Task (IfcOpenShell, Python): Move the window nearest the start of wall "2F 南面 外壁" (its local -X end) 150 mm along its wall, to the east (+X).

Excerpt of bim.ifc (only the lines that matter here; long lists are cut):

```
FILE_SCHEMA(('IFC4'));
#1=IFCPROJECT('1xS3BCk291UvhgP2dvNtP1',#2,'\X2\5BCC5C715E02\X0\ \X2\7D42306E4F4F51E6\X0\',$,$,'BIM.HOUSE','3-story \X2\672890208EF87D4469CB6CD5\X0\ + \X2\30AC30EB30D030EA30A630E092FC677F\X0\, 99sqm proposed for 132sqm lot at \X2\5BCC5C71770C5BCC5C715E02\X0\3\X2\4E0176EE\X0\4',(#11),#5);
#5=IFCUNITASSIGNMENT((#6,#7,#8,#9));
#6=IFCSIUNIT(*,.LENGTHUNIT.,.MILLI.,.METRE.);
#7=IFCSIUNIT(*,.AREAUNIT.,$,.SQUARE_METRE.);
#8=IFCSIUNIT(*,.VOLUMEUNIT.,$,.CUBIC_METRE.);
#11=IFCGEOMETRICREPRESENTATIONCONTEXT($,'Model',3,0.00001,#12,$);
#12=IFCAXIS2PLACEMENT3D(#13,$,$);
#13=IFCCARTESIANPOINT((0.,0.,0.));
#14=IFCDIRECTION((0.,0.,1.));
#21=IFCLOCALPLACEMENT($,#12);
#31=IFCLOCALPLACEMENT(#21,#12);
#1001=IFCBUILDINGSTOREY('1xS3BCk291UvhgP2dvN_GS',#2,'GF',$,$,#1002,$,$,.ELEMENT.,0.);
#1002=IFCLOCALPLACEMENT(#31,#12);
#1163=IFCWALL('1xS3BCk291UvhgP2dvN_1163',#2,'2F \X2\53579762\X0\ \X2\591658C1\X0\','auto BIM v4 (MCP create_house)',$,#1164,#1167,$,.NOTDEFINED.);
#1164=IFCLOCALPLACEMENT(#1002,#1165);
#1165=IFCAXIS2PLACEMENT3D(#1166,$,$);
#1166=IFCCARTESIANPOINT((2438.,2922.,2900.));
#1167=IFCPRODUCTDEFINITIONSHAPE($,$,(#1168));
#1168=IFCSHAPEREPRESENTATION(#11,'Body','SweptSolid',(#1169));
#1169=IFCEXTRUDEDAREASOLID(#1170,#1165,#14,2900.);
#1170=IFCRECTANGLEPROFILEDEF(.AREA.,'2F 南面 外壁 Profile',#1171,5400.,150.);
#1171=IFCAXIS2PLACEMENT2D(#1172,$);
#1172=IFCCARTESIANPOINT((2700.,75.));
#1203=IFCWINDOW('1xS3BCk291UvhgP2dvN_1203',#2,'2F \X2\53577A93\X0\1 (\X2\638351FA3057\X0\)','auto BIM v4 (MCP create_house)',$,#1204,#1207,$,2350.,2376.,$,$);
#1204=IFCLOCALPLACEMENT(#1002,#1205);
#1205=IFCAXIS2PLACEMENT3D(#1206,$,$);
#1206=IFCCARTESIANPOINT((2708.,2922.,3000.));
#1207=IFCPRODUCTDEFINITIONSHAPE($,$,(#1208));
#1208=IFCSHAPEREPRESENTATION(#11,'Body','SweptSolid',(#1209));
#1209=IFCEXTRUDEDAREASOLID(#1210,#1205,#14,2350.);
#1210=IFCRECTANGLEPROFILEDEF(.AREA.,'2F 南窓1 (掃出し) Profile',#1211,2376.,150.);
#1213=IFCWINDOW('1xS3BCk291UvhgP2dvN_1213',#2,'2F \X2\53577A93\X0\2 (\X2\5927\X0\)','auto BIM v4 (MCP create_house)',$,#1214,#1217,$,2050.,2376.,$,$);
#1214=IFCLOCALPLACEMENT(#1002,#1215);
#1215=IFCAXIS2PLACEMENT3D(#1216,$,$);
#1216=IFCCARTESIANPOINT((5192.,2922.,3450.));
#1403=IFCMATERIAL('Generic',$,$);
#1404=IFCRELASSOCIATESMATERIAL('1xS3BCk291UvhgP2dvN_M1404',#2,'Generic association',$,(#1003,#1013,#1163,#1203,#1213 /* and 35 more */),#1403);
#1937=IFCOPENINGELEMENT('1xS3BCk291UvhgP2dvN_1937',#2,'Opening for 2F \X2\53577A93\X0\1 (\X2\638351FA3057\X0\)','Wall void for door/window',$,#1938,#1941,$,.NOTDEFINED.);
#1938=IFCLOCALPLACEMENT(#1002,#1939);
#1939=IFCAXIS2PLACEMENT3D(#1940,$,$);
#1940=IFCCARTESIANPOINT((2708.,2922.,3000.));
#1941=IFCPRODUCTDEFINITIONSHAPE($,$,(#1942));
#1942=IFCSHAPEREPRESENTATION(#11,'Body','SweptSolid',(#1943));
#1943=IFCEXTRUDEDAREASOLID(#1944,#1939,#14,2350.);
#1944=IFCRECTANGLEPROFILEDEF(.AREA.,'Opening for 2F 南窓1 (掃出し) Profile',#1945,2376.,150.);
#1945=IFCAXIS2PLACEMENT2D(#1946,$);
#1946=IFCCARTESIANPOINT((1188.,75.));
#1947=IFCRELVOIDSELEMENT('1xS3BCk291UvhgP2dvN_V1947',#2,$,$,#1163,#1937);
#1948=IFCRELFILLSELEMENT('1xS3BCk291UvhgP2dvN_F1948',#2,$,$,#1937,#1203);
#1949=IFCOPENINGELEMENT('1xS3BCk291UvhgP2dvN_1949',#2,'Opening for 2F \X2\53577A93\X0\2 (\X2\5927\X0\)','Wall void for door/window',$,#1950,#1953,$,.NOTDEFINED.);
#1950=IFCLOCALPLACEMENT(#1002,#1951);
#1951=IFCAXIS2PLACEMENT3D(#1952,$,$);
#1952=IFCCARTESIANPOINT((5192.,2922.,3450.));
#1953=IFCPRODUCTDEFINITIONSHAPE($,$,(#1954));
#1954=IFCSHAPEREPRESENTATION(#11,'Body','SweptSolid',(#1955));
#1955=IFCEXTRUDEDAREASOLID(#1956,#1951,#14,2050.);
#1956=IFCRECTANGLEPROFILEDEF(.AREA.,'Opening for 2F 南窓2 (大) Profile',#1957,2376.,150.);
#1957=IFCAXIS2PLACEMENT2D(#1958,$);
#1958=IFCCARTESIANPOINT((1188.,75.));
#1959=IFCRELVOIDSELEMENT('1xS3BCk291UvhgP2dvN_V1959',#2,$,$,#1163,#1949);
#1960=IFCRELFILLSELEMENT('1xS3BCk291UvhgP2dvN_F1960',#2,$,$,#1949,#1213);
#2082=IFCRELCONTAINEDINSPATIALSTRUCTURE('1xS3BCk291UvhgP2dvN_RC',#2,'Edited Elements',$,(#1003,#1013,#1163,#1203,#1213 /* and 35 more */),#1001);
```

```python
import ifcopenshell
import ifcopenshell.api.geometry
import ifcopenshell.util.placement

model = ifcopenshell.open("bim.ifc")

window = model.by_guid("1xS3BCk291UvhgP2dvN_1203")
opening = window.FillsVoids[0].RelatingOpeningElement
wall = opening.VoidsElements[0].RelatingBuildingElement

wall_matrix = ifcopenshell.util.placement.get_local_placement(wall.ObjectPlacement)
shift = wall_matrix[:3, 0] * 150.0
before = ifcopenshell.util.placement.get_local_placement(window.ObjectPlacement)[:3, 3].copy()

# The window is not placed relative to its opening, so move both.
for product in (opening, window):
    matrix = ifcopenshell.util.placement.get_local_placement(product.ObjectPlacement)
    matrix[:3, 3] += shift
    ifcopenshell.api.geometry.edit_object_placement(model, product=product, matrix=matrix, is_si=False)

after = ifcopenshell.util.placement.get_local_placement(window.ObjectPlacement)[:3, 3]
print("window moved by", (after - before).round(3) + 0.0)

model.write("bim_rev.ifc")
```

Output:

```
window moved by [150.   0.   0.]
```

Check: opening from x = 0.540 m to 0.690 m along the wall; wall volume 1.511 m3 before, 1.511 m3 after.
